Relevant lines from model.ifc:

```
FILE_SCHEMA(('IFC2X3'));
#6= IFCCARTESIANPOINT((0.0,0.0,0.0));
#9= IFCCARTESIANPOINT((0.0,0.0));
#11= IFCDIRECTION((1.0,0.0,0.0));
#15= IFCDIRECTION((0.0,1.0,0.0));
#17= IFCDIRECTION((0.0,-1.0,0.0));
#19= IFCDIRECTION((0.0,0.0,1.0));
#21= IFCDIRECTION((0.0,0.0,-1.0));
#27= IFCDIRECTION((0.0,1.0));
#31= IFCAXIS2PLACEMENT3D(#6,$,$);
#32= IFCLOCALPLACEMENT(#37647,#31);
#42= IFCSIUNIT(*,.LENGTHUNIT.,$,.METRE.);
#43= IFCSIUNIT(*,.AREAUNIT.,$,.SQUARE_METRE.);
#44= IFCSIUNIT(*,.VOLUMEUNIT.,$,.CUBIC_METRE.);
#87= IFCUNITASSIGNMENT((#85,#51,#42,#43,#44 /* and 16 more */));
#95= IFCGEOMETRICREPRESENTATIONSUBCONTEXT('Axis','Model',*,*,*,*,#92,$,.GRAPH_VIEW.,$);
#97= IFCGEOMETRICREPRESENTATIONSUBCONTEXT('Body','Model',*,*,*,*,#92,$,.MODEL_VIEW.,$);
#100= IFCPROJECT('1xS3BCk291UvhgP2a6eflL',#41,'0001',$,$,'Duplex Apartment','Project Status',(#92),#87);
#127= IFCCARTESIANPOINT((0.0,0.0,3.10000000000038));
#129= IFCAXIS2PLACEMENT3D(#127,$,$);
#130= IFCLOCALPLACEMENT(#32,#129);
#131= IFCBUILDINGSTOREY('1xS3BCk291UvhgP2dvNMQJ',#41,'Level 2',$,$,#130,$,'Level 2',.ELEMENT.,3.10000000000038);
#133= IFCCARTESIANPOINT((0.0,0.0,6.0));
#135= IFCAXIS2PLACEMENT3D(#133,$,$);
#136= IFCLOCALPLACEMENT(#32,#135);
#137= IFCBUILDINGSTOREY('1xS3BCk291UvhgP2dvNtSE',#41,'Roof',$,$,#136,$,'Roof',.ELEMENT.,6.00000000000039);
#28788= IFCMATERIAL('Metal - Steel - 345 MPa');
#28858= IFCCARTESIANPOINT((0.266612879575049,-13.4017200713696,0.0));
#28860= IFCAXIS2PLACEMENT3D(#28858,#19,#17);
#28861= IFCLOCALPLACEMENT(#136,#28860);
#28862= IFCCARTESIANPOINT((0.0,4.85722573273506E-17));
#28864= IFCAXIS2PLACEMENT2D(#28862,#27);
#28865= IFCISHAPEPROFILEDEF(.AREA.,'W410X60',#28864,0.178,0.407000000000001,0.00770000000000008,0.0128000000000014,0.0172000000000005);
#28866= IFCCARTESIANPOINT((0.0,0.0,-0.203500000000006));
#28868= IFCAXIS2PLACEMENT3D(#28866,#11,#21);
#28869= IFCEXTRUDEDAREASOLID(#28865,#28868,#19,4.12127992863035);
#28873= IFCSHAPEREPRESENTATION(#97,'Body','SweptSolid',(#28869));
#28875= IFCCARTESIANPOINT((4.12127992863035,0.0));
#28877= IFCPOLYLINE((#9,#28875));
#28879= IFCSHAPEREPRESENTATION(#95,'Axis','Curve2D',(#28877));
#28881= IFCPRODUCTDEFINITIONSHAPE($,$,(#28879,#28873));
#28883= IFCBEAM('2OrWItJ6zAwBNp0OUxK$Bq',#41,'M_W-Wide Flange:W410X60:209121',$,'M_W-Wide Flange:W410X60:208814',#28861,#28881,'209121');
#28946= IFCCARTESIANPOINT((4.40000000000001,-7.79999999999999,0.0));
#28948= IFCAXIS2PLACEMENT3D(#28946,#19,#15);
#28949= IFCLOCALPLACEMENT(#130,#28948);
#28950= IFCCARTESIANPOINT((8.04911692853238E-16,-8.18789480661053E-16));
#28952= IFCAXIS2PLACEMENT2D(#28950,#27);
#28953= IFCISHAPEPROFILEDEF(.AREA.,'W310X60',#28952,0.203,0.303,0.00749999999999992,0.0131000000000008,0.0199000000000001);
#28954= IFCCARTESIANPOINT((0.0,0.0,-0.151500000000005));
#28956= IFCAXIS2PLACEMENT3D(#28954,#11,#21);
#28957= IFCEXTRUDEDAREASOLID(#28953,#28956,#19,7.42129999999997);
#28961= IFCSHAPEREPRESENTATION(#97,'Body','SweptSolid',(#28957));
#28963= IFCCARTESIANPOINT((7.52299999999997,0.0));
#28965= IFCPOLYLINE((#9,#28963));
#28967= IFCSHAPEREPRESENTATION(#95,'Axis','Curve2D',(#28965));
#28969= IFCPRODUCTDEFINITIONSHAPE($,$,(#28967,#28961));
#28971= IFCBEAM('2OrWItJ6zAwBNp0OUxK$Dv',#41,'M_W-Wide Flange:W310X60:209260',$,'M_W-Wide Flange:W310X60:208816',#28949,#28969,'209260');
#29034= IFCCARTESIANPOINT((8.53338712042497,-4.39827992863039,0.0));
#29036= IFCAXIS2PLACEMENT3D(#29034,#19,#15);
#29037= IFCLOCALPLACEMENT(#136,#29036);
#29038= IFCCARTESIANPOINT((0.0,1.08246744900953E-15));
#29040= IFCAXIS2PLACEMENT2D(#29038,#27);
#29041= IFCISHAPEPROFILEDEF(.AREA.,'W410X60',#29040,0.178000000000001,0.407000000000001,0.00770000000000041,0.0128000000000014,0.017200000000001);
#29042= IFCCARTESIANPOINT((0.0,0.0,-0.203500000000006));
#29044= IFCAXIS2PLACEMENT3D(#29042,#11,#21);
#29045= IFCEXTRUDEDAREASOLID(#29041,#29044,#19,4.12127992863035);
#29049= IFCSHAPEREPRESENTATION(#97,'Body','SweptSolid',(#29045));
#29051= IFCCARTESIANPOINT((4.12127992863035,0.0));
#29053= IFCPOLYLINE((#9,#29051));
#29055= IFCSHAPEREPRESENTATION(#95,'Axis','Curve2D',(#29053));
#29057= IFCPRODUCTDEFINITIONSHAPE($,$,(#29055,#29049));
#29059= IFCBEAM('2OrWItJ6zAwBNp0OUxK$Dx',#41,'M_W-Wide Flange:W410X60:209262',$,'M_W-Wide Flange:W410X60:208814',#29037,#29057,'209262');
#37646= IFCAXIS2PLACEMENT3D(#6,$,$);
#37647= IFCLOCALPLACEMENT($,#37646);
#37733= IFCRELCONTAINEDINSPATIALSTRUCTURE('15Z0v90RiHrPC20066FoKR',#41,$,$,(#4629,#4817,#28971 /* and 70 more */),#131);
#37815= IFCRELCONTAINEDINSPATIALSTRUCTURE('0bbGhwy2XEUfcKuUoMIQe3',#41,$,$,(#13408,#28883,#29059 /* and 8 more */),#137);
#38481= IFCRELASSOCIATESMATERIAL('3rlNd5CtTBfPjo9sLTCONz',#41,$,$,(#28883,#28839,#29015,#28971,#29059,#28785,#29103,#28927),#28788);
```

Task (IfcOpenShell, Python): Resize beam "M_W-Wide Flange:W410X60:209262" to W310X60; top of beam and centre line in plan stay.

```python
import ifcopenshell
import ifcopenshell.util.element
import ifcopenshell.util.representation

model = ifcopenshell.open("model.ifc")

member = model.by_id(29059)
source = next(p for p in model.by_type("IfcIShapeProfileDef") if p.ProfileName == "W310X60")

body = ifcopenshell.util.representation.get_representation(member, "Model", "Body")
solid = body.Items[0]
old_profile = solid.SweptArea

# Copy the section's sizes but keep this member's own profile position.
profile = ifcopenshell.util.element.copy(model, source)
# Profiles are centred, so shift by half the change in depth to hold the top.
shift = (old_profile.OverallDepth - profile.OverallDepth) / 2
x, y = old_profile.Position.Location.Coordinates
up = (-1.0, 0.0)  # upwards, in the solid's own plane
location = model.createIfcCartesianPoint((x + up[0] * shift, y + up[1] * shift))
profile.Position = model.createIfcAxis2Placement2D(location, old_profile.Position.RefDirection)
solid.SweptArea = profile
if not model.get_total_inverses(old_profile):
    ifcopenshell.util.element.remove_deep2(model, old_profile)
member.Name = member.Name.replace("W410X60", "W310X60")
member.ObjectType = member.ObjectType.replace("W410X60", "W310X60")

print(solid.SweptArea)

model.write("model_v2.ifc")
```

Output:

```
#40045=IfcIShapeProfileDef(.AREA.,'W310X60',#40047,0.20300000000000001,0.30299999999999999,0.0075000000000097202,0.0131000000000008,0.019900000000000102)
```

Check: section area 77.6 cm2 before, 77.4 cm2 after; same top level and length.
